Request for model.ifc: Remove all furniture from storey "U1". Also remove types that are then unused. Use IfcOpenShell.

First a look at what the model holds.

```python
import ifcopenshell
import ifcopenshell.util.element

model = ifcopenshell.open("model.ifc")
print(model.schema)
storey = next(s for s in model.by_type("IfcBuildingStorey") if s.Name == "U1")
furniture = [e for e in ifcopenshell.util.element.get_decomposition(storey) if e.is_a("IfcFurnishingElement")]
seen = {}
for e in furniture:
    element_type = ifcopenshell.util.element.get_type(e)
    name = element_type.Name if element_type not in (None, e) else None
    seen[name] = seen.get(name, 0) + 1
for name, count in sorted(seen.items(), key=str):
    print(count, "x", name)
```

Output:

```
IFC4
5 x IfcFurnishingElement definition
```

```python
import ifcopenshell
import ifcopenshell.api.root
import ifcopenshell.util.element

model = ifcopenshell.open("model.ifc")

storey = next(s for s in model.by_type("IfcBuildingStorey") if s.Name == "U1")
furniture = [e for e in ifcopenshell.util.element.get_decomposition(storey) if e.is_a("IfcFurnishingElement")]
types = {ifcopenshell.util.element.get_type(e) for e in furniture} - {None, *furniture}

for e in furniture:
    ifcopenshell.api.root.remove_product(model, product=e)
print(len(furniture), "removed")

unused = [t for t in types if not ifcopenshell.util.element.get_types(t)]
for t in unused:
    ifcopenshell.api.root.remove_product(model, product=t)
print(len(unused), "unused types removed")

model.write("model_updated.ifc")
```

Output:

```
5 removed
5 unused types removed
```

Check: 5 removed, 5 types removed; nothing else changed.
